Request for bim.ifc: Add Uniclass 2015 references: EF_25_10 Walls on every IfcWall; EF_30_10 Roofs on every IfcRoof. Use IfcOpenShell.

First a look at what the model holds.

```python
import ifcopenshell

model = ifcopenshell.open("bim.ifc")
print(model.schema)
print("classifications:", [c.Name for c in model.by_type("IfcClassification")])
for ifc_class in ("IfcDoor", "IfcRoof", "IfcStair", "IfcWall", "IfcWindow"):
    print(ifc_class, len(model.by_type(ifc_class)))
```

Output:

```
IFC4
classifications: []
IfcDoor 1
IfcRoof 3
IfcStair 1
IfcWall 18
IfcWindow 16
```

```python
import ifcopenshell
import ifcopenshell.api.classification

model = ifcopenshell.open("bim.ifc")

system = ifcopenshell.api.classification.add_classification(model, classification="Uniclass 2015")

codes = {
    "IfcWall": ("EF_25_10", "Walls"),
    "IfcRoof": ("EF_30_10", "Roofs"),
}
for ifc_class, (code, name) in codes.items():
    products = model.by_type(ifc_class)
    ifcopenshell.api.classification.add_reference(
        model, products=products, classification=system, identification=code, name=name
    )
    print(code, len(products))

model.write("bim_updated.ifc")
```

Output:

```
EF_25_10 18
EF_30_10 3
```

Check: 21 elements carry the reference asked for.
